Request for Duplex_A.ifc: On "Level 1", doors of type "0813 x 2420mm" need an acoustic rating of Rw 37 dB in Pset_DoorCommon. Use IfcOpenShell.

First a look at what the model holds.

```python
import ifcopenshell
import ifcopenshell.util.element

model = ifcopenshell.open("Duplex_A.ifc")
print(model.schema)
storey = next(s for s in model.by_type("IfcBuildingStorey") if s.Name == "Level 1")
doors = [e for e in ifcopenshell.util.element.get_decomposition(storey) if e.is_a("IfcDoor")]
seen = {}
for e in doors:
    element_type = ifcopenshell.util.element.get_type(e)
    key = (element_type.Name if element_type != e and element_type else None, ifcopenshell.util.element.get_pset(e, "Pset_DoorCommon", "AcousticRating"))
    seen[key] = seen.get(key, 0) + 1
for (name, value), count in sorted(seen.items(), key=str):
    print(count, "x", name, "|", value)
```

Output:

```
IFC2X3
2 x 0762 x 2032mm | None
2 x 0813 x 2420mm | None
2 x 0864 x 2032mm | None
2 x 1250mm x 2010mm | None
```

```python
import ifcopenshell
import ifcopenshell.api.pset
import ifcopenshell.util.element

model = ifcopenshell.open("Duplex_A.ifc")

storey = next(s for s in model.by_type("IfcBuildingStorey") if s.Name == "Level 1")
doors = [e for e in ifcopenshell.util.element.get_decomposition(storey) if e.is_a("IfcDoor")]

count = 0
for e in doors:
    element_type = ifcopenshell.util.element.get_type(e)
    if element_type in (None, e) or element_type.Name != "0813 x 2420mm":
        continue
    # add_pset returns the element's existing set when there is one.
    pset = ifcopenshell.api.pset.add_pset(model, product=e, name="Pset_DoorCommon")
    ifcopenshell.api.pset.edit_pset(model, pset=pset, properties={"AcousticRating": "Rw 37 dB"})
    count += 1

print(count, "doors updated")

model.write("Duplex_A_v2.ifc")
```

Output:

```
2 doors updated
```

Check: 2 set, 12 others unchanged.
